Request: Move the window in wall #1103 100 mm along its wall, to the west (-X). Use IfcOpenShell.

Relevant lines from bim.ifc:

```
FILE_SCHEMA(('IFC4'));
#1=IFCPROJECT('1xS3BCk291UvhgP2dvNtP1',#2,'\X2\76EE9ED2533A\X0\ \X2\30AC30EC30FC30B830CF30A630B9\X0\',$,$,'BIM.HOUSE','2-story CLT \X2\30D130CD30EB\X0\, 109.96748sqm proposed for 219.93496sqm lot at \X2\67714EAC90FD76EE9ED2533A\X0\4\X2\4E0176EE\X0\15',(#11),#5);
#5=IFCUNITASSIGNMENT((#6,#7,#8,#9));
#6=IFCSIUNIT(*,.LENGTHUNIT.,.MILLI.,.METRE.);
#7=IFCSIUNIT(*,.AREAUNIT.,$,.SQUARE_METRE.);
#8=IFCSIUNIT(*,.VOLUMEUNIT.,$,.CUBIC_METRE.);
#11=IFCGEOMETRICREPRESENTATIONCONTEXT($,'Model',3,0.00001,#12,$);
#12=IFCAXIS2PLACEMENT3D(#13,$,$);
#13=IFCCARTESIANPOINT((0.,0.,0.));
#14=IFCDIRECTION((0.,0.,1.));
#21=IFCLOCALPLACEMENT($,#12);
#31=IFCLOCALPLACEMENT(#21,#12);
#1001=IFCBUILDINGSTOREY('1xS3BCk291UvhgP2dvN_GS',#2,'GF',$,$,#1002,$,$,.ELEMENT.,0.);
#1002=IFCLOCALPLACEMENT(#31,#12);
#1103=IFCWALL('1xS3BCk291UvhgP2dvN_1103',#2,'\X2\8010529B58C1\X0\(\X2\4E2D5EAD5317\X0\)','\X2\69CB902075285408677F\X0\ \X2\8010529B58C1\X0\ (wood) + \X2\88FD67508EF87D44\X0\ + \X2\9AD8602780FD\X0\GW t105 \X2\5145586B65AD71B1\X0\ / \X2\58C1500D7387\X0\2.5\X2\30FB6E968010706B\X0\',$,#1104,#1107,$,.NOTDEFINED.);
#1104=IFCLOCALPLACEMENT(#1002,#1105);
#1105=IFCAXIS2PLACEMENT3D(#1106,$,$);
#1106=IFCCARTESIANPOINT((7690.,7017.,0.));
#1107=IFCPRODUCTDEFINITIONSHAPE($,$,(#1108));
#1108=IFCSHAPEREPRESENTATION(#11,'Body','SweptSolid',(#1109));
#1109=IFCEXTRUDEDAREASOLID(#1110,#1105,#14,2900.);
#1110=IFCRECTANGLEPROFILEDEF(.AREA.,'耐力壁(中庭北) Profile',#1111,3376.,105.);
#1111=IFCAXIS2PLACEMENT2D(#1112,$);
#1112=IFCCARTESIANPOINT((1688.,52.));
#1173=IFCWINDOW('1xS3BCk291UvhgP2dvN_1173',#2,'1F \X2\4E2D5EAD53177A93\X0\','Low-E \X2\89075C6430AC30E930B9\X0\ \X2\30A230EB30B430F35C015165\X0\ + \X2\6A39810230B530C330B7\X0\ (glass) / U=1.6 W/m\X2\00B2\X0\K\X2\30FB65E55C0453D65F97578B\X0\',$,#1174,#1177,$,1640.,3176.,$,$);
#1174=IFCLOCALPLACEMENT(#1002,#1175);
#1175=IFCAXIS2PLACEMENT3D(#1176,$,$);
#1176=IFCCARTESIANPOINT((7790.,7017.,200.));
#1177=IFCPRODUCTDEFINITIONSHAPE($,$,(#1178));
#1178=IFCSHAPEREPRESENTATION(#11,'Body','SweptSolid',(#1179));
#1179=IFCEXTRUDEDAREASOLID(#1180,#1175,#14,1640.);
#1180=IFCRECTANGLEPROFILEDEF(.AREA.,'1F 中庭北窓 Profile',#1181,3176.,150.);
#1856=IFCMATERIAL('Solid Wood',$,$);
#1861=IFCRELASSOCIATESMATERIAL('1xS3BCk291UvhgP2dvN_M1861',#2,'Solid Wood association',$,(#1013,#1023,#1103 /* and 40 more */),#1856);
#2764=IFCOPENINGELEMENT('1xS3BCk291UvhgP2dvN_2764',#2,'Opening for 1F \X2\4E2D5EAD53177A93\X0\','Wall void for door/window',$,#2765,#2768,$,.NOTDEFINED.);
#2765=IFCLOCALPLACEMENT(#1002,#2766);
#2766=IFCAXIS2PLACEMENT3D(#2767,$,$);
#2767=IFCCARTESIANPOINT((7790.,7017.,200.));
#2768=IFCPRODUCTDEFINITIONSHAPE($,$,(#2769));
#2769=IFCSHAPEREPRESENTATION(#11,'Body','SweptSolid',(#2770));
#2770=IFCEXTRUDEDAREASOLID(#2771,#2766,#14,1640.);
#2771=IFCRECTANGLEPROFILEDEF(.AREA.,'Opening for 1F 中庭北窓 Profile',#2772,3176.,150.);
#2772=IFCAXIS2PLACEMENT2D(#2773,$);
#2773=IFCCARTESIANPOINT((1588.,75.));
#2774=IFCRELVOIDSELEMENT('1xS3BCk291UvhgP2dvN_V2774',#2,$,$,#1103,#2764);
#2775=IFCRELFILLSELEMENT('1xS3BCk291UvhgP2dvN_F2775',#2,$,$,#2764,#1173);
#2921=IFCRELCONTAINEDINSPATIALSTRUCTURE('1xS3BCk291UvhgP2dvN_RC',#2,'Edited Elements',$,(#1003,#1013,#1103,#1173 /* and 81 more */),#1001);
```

```python
import ifcopenshell
import ifcopenshell.api.geometry
import ifcopenshell.util.placement
import ifcopenshell.util.unit

model = ifcopenshell.open("bim.ifc")
unit_scale = ifcopenshell.util.unit.calculate_unit_scale(model)

window = model.by_guid("1xS3BCk291UvhgP2dvN_1173")
opening = window.FillsVoids[0].RelatingOpeningElement
wall = opening.VoidsElements[0].RelatingBuildingElement

wall_matrix = ifcopenshell.util.placement.get_local_placement(wall.ObjectPlacement)
shift = wall_matrix[:3, 0] * -0.1 / unit_scale
before = ifcopenshell.util.placement.get_local_placement(window.ObjectPlacement)[:3, 3].copy()

# The window is not placed relative to its opening, so move both.
for product in (opening, window):
    matrix = ifcopenshell.util.placement.get_local_placement(product.ObjectPlacement)
    matrix[:3, 3] += shift
    ifcopenshell.api.geometry.edit_object_placement(model, product=product, matrix=matrix, is_si=False)

after = ifcopenshell.util.placement.get_local_placement(window.ObjectPlacement)[:3, 3]
print("window moved by", (after - before).round(3) + 0.0)

model.write("bim_updated.ifc")
```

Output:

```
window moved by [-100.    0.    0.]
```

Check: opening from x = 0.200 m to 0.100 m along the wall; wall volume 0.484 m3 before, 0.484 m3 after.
